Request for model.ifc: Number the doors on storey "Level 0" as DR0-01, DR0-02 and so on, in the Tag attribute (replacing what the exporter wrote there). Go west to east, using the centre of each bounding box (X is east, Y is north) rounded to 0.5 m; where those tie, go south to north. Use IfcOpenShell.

First a look at what the model holds.

```python
import ifcopenshell
import ifcopenshell.util.element
import ifcopenshell.util.placement

model = ifcopenshell.open("model.ifc")
print(model.schema)
storey = next(s for s in model.by_type("IfcBuildingStorey") if s.Name == "Level 0")
doors = [e for e in ifcopenshell.util.element.get_decomposition(storey) if e.is_a("IfcDoor")]
for e in sorted(doors, key=lambda e: e.id()):
    origin = ifcopenshell.util.placement.get_local_placement(e.ObjectPlacement)[:3, 3]
    print(e.id(), e.Tag, e.Name, origin.round(2) + 0.0, sep=" | ")
```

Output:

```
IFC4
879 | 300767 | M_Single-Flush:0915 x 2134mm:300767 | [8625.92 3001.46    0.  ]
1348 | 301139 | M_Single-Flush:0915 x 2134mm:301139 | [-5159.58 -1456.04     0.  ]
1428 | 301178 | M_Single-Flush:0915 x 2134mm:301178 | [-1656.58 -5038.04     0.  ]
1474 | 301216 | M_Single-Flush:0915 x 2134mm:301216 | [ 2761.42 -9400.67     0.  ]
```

```python
import ifcopenshell
import ifcopenshell.geom
import ifcopenshell.util.element
import ifcopenshell.util.shape

model = ifcopenshell.open("model.ifc")
settings = ifcopenshell.geom.settings()
settings.set("use-world-coords", True)


def centre(element):
    shape = ifcopenshell.geom.create_shape(settings, element)
    return ifcopenshell.util.shape.get_bbox_centroid(shape.geometry)


storey = next(s for s in model.by_type("IfcBuildingStorey") if s.Name == "Level 0")
doors = [e for e in ifcopenshell.util.element.get_decomposition(storey) if e.is_a("IfcDoor")]

# Insertion points can sit at a corner or the storey origin, so sort by the geometry (in metres).
centres = {e: centre(e) for e in doors}
doors.sort(key=lambda e: (round(centres[e][0] / 0.5), centres[e][1]))

for i, e in enumerate(doors, start=1):
    number = f"DR0-{i:02d}"
    e.Tag = number
    print(e.id(), number)

model.write("model-out.ifc")
```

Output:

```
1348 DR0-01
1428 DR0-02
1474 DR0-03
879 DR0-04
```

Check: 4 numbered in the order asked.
